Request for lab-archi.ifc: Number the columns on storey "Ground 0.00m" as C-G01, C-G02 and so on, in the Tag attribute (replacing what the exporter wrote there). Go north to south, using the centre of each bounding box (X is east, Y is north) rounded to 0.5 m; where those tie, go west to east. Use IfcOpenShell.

First a look at what the model holds.

```python
import ifcopenshell
import ifcopenshell.util.element
import ifcopenshell.util.placement

model = ifcopenshell.open("lab-archi.ifc")
print(model.schema)
storey = next(s for s in model.by_type("IfcBuildingStorey") if s.Name == "Ground 0.00m")
columns = [e for e in ifcopenshell.util.element.get_decomposition(storey) if e.is_a("IfcColumn")]
for e in sorted(columns, key=lambda e: e.id()):
    origin = ifcopenshell.util.placement.get_local_placement(e.ObjectPlacement)[:3, 3]
    print(e.id(), e.Tag, e.Name, origin.round(2) + 0.0, sep=" | ")
```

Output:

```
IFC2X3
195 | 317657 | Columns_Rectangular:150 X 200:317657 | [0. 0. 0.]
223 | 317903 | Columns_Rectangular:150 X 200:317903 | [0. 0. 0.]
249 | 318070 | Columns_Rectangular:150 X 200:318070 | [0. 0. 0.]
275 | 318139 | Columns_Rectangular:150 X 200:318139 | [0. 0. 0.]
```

```python
import ifcopenshell
import ifcopenshell.geom
import ifcopenshell.util.element
import ifcopenshell.util.shape

model = ifcopenshell.open("lab-archi.ifc")
settings = ifcopenshell.geom.settings()
settings.set("use-world-coords", True)


def centre(element):
    shape = ifcopenshell.geom.create_shape(settings, element)
    return ifcopenshell.util.shape.get_bbox_centroid(shape.geometry)


storey = next(s for s in model.by_type("IfcBuildingStorey") if s.Name == "Ground 0.00m")
columns = [e for e in ifcopenshell.util.element.get_decomposition(storey) if e.is_a("IfcColumn")]

# Insertion points can sit at a corner or the storey origin, so sort by the geometry (in metres).
centres = {e: centre(e) for e in columns}
columns.sort(key=lambda e: (-round(centres[e][1] / 0.5), centres[e][0]))

for i, e in enumerate(columns, start=1):
    number = f"C-G{i:02d}"
    e.Tag = number
    print(e.id(), number)

model.write("lab-archi-out.ifc")
```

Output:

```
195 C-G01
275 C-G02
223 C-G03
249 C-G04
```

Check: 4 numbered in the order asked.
